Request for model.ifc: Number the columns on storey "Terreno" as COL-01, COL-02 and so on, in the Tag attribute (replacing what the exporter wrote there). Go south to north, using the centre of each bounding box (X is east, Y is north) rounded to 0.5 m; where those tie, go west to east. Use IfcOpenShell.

First a look at what the model holds.

```python
import ifcopenshell
import ifcopenshell.util.element
import ifcopenshell.util.placement

model = ifcopenshell.open("model.ifc")
print(model.schema)
storey = next(s for s in model.by_type("IfcBuildingStorey") if s.Name == "Terreno")
columns = [e for e in ifcopenshell.util.element.get_decomposition(storey) if e.is_a("IfcColumn")]
for e in sorted(columns, key=lambda e: e.id()):
    origin = ifcopenshell.util.placement.get_local_placement(e.ObjectPlacement)[:3, 3]
    print(e.id(), e.Tag, e.Name, origin.round(2) + 0.0, sep=" | ")
```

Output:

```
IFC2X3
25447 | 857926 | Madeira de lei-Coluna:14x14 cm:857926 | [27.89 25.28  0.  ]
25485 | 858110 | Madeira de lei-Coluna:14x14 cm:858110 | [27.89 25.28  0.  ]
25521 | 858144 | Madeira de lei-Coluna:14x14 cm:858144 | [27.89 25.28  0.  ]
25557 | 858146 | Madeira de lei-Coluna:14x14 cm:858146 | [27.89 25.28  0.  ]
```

```python
import ifcopenshell
import ifcopenshell.geom
import ifcopenshell.util.element
import ifcopenshell.util.shape

model = ifcopenshell.open("model.ifc")
settings = ifcopenshell.geom.settings()
settings.set("use-world-coords", True)


def centre(element):
    shape = ifcopenshell.geom.create_shape(settings, element)
    return ifcopenshell.util.shape.get_bbox_centroid(shape.geometry)


storey = next(s for s in model.by_type("IfcBuildingStorey") if s.Name == "Terreno")
columns = [e for e in ifcopenshell.util.element.get_decomposition(storey) if e.is_a("IfcColumn")]

# Insertion points can sit at a corner or the storey origin, so sort by the geometry (in metres).
centres = {e: centre(e) for e in columns}
columns.sort(key=lambda e: (round(centres[e][1] / 0.5), centres[e][0]))

for i, e in enumerate(columns, start=1):
    number = f"COL-{i:02d}"
    e.Tag = number
    print(e.id(), number)

model.write("model-out.ifc")
```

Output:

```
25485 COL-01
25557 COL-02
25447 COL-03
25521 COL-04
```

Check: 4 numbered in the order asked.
